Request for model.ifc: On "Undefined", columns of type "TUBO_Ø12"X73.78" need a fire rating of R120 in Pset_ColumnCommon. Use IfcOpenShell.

First a look at what the model holds.

```python
import ifcopenshell
import ifcopenshell.util.element

model = ifcopenshell.open("model.ifc")
print(model.schema)
storey = next(s for s in model.by_type("IfcBuildingStorey") if s.Name == "Undefined")
columns = [e for e in ifcopenshell.util.element.get_decomposition(storey) if e.is_a("IfcColumn")]
seen = {}
for e in columns:
    element_type = ifcopenshell.util.element.get_type(e)
    key = (element_type.Name if element_type != e and element_type else None, ifcopenshell.util.element.get_pset(e, "Pset_ColumnCommon", "FireRating"))
    seen[key] = seen.get(key, 0) + 1
for (name, value), count in sorted(seen.items(), key=str):
    print(count, "x", name, "|", value)
```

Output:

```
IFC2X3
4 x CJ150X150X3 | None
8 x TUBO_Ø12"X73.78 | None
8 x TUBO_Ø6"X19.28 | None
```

```python
import ifcopenshell
import ifcopenshell.api.pset
import ifcopenshell.util.element

model = ifcopenshell.open("model.ifc")

storey = next(s for s in model.by_type("IfcBuildingStorey") if s.Name == "Undefined")
columns = [e for e in ifcopenshell.util.element.get_decomposition(storey) if e.is_a("IfcColumn")]

count = 0
for e in columns:
    element_type = ifcopenshell.util.element.get_type(e)
    if element_type in (None, e) or element_type.Name != 'TUBO_Ø12"X73.78':
        continue
    found = ifcopenshell.util.element.get_pset(e, "Pset_ColumnCommon", should_inherit=False)
    if found:
        pset = model.by_id(found["id"])
        if len(ifcopenshell.util.element.get_elements_by_pset(pset)) > 1:
            pset = ifcopenshell.api.pset.unshare_pset(model, products=[e], pset=pset)[0]
    else:
        pset = ifcopenshell.api.pset.add_pset(model, product=e, name="Pset_ColumnCommon")
    ifcopenshell.api.pset.edit_pset(model, pset=pset, properties={"FireRating": "R120"})
    count += 1

print(count, "columns updated")

model.write("model_rev.ifc")
```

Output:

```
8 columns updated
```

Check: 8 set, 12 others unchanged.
